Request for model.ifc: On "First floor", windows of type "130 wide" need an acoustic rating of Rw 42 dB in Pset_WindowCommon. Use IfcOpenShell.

First a look at what the model holds.

```python
import ifcopenshell
import ifcopenshell.util.element

model = ifcopenshell.open("model.ifc")
print(model.schema)
storey = next(s for s in model.by_type("IfcBuildingStorey") if s.Name == "First floor")
windows = [e for e in ifcopenshell.util.element.get_decomposition(storey) if e.is_a("IfcWindow")]
seen = {}
for e in windows:
    element_type = ifcopenshell.util.element.get_type(e)
    key = (element_type.Name if element_type != e and element_type else None, ifcopenshell.util.element.get_pset(e, "Pset_WindowCommon", "AcousticRating"))
    seen[key] = seen.get(key, 0) + 1
for (name, value), count in sorted(seen.items(), key=str):
    print(count, "x", name, "|", value)
```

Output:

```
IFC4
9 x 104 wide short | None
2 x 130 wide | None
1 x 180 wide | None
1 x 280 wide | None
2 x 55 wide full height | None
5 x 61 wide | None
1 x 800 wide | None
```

```python
import ifcopenshell
import ifcopenshell.api.pset
import ifcopenshell.util.element

model = ifcopenshell.open("model.ifc")

storey = next(s for s in model.by_type("IfcBuildingStorey") if s.Name == "First floor")
windows = [e for e in ifcopenshell.util.element.get_decomposition(storey) if e.is_a("IfcWindow")]

count = 0
for e in windows:
    element_type = ifcopenshell.util.element.get_type(e)
    if element_type in (None, e) or element_type.Name != "130 wide":
        continue
    # add_pset returns the element's existing set when there is one.
    pset = ifcopenshell.api.pset.add_pset(model, product=e, name="Pset_WindowCommon")
    ifcopenshell.api.pset.edit_pset(model, pset=pset, properties={"AcousticRating": "Rw 42 dB"})
    count += 1

print(count, "windows updated")

model.write("model_rev.ifc")
```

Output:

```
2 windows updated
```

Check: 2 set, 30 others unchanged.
